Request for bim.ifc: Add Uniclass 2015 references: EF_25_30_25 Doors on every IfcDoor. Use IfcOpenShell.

First a look at what the model holds.

```python
import ifcopenshell

model = ifcopenshell.open("bim.ifc")
print(model.schema)
print("classifications:", [c.Name for c in model.by_type("IfcClassification")])
for ifc_class in ("IfcDoor", "IfcRoof", "IfcStair", "IfcWall", "IfcWindow"):
    print(ifc_class, len(model.by_type(ifc_class)))
```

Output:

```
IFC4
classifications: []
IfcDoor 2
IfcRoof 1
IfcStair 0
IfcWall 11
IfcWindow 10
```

```python
import ifcopenshell
import ifcopenshell.api.classification

model = ifcopenshell.open("bim.ifc")

system = ifcopenshell.api.classification.add_classification(model, classification="Uniclass 2015")

codes = {
    "IfcDoor": ("EF_25_30_25", "Doors"),
}
for ifc_class, (code, name) in codes.items():
    products = model.by_type(ifc_class)
    ifcopenshell.api.classification.add_reference(
        model, products=products, classification=system, identification=code, name=name
    )
    print(code, len(products))

model.write("bim_v2.ifc")
```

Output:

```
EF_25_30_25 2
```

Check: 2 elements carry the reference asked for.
